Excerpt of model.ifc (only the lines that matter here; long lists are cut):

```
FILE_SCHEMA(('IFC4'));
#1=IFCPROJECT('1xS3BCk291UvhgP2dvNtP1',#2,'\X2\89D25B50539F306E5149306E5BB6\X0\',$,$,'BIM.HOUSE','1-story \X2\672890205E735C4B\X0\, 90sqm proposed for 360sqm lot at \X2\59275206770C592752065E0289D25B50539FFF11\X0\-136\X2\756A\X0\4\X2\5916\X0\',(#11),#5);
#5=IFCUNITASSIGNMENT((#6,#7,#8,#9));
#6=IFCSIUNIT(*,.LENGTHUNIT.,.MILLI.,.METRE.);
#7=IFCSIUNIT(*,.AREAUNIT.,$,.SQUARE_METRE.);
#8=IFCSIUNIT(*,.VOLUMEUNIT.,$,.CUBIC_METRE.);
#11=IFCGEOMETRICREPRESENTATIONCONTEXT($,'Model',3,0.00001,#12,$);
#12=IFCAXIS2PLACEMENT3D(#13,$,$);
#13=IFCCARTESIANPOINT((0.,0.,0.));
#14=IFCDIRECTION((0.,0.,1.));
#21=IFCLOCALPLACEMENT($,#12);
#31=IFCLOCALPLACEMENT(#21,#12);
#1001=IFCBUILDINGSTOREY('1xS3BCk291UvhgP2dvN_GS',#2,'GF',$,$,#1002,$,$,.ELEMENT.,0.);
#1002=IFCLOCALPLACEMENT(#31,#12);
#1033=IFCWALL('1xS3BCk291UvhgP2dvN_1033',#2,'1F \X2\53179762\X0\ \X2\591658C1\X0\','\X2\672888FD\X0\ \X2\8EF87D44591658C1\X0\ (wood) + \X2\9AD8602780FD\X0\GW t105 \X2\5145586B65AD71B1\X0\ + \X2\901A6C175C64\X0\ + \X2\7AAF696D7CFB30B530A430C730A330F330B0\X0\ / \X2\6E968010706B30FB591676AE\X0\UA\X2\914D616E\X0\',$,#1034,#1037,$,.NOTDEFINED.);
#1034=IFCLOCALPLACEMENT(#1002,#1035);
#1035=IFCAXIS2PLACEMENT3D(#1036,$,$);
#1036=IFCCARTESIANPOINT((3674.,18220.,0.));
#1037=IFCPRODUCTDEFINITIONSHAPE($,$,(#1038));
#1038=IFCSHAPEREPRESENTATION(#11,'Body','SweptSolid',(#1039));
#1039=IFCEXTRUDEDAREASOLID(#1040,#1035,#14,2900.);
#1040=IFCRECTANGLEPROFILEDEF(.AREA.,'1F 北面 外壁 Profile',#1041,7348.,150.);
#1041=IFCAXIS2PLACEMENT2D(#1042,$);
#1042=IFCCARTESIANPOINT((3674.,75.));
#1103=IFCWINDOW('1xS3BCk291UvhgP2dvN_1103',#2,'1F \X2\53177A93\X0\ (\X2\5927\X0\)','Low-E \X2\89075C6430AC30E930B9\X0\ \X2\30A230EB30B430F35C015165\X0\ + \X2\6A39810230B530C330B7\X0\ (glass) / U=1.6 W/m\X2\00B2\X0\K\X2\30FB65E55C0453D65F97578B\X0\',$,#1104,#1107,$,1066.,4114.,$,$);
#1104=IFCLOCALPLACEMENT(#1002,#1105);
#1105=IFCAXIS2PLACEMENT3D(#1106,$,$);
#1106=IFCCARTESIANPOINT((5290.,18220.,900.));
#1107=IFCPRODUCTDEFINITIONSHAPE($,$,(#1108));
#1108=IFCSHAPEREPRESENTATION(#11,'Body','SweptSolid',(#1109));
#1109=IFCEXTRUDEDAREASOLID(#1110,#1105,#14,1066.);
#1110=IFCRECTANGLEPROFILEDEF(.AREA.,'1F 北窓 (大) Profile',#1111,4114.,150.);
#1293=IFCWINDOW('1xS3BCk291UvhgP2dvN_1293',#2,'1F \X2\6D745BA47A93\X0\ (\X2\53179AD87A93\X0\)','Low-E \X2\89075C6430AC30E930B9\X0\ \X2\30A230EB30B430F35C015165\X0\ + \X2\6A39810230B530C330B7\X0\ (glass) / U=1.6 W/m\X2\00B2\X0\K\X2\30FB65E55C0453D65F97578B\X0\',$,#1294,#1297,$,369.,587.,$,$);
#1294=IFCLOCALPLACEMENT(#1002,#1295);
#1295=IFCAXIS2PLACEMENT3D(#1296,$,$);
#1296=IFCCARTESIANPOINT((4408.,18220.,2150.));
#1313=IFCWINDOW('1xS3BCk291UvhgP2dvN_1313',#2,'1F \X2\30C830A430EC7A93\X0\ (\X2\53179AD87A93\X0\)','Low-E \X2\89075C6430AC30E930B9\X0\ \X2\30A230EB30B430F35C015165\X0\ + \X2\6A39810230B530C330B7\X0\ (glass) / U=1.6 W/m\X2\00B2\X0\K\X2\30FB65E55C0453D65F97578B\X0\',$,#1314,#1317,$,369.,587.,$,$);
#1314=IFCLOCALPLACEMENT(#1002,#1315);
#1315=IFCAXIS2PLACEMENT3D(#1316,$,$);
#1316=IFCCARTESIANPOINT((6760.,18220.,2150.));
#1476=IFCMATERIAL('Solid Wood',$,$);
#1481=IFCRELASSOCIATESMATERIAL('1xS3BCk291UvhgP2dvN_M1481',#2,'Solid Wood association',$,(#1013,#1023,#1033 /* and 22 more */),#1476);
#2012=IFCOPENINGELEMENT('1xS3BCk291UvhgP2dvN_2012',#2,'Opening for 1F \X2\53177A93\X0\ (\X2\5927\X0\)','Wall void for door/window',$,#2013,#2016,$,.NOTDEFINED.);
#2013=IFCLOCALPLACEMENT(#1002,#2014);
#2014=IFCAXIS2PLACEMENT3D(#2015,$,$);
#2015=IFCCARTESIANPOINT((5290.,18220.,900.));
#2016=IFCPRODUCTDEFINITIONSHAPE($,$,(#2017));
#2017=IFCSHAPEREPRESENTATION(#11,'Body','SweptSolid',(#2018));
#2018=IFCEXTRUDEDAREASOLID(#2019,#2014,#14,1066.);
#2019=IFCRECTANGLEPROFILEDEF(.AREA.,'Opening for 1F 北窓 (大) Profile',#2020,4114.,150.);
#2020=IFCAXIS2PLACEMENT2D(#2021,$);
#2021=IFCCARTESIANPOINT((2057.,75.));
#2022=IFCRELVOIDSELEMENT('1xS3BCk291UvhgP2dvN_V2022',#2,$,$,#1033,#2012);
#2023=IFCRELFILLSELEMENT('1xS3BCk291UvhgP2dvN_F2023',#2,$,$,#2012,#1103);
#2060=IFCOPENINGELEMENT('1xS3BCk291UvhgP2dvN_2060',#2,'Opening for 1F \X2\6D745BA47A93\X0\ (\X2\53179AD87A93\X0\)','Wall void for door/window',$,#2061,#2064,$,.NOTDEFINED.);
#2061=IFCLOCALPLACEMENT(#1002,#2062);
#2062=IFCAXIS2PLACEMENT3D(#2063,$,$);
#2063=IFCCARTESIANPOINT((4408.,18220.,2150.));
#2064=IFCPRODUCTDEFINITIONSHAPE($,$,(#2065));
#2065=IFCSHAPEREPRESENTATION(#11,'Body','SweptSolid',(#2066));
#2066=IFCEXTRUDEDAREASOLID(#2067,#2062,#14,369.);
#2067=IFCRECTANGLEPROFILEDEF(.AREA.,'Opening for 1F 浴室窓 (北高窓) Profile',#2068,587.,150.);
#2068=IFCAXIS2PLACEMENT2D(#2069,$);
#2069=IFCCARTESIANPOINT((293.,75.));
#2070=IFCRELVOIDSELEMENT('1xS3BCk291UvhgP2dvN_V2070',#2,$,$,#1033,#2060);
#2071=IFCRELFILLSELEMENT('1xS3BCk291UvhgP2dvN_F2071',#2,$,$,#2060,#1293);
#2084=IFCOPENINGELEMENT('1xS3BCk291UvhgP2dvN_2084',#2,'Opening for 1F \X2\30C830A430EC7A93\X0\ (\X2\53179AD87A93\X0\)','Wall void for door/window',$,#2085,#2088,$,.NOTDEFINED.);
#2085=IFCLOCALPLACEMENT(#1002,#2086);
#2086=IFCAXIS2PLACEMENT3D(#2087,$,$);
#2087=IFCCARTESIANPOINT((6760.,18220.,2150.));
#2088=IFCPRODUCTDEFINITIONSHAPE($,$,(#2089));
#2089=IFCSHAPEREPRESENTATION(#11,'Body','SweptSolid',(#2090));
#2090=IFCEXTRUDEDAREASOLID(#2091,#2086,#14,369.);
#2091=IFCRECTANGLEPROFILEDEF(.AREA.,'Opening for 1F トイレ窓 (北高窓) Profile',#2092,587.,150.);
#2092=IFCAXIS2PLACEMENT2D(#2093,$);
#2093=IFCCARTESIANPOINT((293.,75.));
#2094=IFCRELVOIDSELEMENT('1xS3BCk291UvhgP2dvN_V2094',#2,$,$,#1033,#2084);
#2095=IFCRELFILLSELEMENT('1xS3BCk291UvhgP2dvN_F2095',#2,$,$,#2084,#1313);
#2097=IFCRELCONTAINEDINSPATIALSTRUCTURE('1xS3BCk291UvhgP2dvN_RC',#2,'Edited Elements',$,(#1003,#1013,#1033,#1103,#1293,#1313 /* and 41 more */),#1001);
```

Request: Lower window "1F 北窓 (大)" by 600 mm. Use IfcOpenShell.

```python
import numpy as np
import ifcopenshell
import ifcopenshell.api.geometry
import ifcopenshell.util.placement
import ifcopenshell.util.unit

model = ifcopenshell.open("model.ifc")
unit_scale = ifcopenshell.util.unit.calculate_unit_scale(model)

window = model.by_id(1103)
opening = window.FillsVoids[0].RelatingOpeningElement
dz = -0.6 / unit_scale

shift = np.array([0.0, 0.0, dz])
# The window is not placed relative to its opening, so move both.
for product in (opening, window):
    matrix = ifcopenshell.util.placement.get_local_placement(product.ObjectPlacement)
    matrix[:3, 3] += shift
    ifcopenshell.api.geometry.edit_object_placement(model, product=product, matrix=matrix, is_si=False)

print(f"moved by {dz * unit_scale:+.3f} m")

model.write("model_v2.ifc")
```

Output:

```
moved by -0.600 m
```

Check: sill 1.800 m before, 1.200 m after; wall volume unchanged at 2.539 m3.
